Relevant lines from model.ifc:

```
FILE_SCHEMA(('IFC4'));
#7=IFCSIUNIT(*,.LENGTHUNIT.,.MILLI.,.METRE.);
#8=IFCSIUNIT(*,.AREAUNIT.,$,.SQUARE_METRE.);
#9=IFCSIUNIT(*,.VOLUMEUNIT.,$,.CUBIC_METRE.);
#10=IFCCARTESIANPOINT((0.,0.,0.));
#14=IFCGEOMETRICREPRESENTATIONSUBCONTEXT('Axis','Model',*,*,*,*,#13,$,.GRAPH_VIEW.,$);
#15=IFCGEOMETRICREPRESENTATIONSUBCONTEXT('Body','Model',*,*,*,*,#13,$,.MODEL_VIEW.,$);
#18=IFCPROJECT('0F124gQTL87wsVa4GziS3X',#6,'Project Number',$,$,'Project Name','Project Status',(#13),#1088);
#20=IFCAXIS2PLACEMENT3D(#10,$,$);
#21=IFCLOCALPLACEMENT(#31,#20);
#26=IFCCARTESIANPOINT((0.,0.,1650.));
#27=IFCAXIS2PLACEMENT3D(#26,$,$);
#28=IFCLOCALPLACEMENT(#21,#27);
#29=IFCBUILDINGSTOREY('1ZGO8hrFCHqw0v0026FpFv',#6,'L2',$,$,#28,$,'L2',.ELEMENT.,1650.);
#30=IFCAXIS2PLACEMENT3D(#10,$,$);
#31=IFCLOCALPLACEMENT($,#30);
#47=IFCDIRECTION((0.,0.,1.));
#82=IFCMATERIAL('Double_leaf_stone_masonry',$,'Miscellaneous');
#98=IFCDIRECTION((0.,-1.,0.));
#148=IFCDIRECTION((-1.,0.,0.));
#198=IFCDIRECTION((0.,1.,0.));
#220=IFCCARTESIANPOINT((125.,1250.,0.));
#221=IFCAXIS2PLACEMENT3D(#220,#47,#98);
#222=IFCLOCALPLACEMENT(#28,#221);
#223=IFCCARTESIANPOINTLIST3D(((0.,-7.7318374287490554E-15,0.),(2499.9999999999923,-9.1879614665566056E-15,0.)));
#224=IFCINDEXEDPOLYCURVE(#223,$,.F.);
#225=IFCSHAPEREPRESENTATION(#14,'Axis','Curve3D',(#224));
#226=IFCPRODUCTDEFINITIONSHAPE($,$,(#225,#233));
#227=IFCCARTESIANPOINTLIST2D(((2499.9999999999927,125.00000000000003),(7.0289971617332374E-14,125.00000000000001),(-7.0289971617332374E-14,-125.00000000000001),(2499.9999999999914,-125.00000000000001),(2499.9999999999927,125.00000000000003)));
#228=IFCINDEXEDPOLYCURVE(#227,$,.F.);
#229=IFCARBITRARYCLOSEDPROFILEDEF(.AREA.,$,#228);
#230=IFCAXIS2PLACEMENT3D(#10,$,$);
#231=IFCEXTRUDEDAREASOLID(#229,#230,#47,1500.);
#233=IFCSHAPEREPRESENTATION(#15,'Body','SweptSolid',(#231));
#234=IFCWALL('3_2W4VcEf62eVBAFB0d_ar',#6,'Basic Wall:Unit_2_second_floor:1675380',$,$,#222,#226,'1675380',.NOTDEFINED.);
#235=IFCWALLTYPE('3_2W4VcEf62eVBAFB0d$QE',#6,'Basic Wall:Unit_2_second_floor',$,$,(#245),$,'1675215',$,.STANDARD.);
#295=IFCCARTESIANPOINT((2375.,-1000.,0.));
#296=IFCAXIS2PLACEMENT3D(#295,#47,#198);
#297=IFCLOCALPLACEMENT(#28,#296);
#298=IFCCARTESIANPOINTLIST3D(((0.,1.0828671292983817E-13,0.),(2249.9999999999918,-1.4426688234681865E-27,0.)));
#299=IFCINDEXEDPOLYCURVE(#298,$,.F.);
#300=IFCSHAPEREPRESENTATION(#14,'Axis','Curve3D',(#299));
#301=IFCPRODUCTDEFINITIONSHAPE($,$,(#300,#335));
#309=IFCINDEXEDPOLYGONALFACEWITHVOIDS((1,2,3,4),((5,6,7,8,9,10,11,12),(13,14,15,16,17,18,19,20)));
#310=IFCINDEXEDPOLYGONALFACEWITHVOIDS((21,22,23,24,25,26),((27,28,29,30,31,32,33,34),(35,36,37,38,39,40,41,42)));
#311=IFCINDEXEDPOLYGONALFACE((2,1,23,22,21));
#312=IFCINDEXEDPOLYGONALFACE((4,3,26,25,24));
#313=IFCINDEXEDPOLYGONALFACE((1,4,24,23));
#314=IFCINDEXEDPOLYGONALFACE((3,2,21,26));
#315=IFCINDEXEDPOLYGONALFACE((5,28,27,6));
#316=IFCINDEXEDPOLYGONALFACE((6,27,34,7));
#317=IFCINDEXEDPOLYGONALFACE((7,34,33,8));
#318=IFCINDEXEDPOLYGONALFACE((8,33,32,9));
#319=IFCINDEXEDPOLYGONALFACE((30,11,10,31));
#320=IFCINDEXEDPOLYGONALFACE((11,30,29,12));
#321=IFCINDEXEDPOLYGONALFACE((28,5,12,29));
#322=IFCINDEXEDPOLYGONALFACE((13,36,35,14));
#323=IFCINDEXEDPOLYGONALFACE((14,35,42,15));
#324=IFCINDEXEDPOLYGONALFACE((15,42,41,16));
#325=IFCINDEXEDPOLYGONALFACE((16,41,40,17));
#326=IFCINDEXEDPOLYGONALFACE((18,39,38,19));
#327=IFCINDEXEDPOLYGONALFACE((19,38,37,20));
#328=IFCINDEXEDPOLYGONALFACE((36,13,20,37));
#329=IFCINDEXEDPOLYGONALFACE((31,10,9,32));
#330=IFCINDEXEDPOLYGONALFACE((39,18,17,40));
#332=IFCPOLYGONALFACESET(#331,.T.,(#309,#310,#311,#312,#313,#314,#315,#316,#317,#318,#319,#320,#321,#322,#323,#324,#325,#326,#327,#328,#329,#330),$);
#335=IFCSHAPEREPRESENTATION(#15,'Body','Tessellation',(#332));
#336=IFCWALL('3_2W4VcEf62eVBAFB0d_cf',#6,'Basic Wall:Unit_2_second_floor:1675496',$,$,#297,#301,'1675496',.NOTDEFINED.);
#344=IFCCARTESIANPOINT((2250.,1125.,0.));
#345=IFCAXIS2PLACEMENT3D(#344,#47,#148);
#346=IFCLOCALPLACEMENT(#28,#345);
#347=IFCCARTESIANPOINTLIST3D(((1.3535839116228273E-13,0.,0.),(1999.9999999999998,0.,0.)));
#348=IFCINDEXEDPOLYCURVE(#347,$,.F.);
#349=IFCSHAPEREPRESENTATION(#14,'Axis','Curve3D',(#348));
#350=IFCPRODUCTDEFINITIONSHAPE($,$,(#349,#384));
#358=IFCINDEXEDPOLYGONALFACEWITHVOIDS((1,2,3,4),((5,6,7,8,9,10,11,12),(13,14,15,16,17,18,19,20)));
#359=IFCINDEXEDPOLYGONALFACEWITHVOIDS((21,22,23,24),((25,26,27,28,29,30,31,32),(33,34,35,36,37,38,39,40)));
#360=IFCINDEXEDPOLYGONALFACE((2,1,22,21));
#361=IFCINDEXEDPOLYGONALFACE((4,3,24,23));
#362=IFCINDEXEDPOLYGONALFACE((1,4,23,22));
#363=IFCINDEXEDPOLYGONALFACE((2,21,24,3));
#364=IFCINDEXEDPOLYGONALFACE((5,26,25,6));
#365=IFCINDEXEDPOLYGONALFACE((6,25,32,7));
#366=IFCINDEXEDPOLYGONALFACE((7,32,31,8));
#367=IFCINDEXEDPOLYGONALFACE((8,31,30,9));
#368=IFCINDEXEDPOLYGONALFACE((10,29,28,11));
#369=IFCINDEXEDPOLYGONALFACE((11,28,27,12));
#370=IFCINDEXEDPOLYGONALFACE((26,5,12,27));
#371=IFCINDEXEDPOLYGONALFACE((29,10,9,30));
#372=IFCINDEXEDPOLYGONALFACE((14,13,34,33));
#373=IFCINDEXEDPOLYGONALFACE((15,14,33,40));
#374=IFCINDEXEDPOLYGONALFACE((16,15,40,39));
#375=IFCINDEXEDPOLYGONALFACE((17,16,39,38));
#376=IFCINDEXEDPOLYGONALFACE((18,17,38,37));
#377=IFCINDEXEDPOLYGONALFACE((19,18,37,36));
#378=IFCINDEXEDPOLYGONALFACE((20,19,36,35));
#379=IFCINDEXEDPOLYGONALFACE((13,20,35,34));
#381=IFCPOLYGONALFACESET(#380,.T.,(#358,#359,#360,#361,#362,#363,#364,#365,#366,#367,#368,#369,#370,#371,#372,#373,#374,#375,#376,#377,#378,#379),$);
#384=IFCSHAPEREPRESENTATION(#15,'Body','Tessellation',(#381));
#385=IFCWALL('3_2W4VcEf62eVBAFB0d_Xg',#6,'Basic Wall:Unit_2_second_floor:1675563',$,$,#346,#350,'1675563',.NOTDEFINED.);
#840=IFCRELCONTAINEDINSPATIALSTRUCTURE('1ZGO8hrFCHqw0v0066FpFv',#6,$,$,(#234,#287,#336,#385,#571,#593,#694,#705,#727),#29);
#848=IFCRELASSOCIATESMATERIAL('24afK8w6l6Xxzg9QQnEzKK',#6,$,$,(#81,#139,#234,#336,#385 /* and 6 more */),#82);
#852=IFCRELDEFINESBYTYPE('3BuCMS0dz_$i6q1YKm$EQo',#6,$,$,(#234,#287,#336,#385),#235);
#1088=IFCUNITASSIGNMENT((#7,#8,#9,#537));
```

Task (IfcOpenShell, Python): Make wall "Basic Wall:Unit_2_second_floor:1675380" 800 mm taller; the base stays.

```python
import ifcopenshell
import ifcopenshell.geom
import ifcopenshell.util.representation
import ifcopenshell.util.shape

model = ifcopenshell.open("model.ifc")
settings = ifcopenshell.geom.settings()


def volume(element):
    """Net volume in cubic metres, openings subtracted."""
    shape = ifcopenshell.geom.create_shape(settings, element)
    return ifcopenshell.util.shape.get_volume(shape.geometry)


wall = model.by_guid("3_2W4VcEf62eVBAFB0d_ar")
before = volume(wall)

body = ifcopenshell.util.representation.get_representation(wall, "Model", "Body")
solid = body.Items[0]
old_height = solid.Depth
solid.Depth += 800.0
after = volume(wall)

print(f"height {old_height:g} -> {solid.Depth:g}, volume {before:.3f} -> {after:.3f} m3")

model.write("model_updated.ifc")
```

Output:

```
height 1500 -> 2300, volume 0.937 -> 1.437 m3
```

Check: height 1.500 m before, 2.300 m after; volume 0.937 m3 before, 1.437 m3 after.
